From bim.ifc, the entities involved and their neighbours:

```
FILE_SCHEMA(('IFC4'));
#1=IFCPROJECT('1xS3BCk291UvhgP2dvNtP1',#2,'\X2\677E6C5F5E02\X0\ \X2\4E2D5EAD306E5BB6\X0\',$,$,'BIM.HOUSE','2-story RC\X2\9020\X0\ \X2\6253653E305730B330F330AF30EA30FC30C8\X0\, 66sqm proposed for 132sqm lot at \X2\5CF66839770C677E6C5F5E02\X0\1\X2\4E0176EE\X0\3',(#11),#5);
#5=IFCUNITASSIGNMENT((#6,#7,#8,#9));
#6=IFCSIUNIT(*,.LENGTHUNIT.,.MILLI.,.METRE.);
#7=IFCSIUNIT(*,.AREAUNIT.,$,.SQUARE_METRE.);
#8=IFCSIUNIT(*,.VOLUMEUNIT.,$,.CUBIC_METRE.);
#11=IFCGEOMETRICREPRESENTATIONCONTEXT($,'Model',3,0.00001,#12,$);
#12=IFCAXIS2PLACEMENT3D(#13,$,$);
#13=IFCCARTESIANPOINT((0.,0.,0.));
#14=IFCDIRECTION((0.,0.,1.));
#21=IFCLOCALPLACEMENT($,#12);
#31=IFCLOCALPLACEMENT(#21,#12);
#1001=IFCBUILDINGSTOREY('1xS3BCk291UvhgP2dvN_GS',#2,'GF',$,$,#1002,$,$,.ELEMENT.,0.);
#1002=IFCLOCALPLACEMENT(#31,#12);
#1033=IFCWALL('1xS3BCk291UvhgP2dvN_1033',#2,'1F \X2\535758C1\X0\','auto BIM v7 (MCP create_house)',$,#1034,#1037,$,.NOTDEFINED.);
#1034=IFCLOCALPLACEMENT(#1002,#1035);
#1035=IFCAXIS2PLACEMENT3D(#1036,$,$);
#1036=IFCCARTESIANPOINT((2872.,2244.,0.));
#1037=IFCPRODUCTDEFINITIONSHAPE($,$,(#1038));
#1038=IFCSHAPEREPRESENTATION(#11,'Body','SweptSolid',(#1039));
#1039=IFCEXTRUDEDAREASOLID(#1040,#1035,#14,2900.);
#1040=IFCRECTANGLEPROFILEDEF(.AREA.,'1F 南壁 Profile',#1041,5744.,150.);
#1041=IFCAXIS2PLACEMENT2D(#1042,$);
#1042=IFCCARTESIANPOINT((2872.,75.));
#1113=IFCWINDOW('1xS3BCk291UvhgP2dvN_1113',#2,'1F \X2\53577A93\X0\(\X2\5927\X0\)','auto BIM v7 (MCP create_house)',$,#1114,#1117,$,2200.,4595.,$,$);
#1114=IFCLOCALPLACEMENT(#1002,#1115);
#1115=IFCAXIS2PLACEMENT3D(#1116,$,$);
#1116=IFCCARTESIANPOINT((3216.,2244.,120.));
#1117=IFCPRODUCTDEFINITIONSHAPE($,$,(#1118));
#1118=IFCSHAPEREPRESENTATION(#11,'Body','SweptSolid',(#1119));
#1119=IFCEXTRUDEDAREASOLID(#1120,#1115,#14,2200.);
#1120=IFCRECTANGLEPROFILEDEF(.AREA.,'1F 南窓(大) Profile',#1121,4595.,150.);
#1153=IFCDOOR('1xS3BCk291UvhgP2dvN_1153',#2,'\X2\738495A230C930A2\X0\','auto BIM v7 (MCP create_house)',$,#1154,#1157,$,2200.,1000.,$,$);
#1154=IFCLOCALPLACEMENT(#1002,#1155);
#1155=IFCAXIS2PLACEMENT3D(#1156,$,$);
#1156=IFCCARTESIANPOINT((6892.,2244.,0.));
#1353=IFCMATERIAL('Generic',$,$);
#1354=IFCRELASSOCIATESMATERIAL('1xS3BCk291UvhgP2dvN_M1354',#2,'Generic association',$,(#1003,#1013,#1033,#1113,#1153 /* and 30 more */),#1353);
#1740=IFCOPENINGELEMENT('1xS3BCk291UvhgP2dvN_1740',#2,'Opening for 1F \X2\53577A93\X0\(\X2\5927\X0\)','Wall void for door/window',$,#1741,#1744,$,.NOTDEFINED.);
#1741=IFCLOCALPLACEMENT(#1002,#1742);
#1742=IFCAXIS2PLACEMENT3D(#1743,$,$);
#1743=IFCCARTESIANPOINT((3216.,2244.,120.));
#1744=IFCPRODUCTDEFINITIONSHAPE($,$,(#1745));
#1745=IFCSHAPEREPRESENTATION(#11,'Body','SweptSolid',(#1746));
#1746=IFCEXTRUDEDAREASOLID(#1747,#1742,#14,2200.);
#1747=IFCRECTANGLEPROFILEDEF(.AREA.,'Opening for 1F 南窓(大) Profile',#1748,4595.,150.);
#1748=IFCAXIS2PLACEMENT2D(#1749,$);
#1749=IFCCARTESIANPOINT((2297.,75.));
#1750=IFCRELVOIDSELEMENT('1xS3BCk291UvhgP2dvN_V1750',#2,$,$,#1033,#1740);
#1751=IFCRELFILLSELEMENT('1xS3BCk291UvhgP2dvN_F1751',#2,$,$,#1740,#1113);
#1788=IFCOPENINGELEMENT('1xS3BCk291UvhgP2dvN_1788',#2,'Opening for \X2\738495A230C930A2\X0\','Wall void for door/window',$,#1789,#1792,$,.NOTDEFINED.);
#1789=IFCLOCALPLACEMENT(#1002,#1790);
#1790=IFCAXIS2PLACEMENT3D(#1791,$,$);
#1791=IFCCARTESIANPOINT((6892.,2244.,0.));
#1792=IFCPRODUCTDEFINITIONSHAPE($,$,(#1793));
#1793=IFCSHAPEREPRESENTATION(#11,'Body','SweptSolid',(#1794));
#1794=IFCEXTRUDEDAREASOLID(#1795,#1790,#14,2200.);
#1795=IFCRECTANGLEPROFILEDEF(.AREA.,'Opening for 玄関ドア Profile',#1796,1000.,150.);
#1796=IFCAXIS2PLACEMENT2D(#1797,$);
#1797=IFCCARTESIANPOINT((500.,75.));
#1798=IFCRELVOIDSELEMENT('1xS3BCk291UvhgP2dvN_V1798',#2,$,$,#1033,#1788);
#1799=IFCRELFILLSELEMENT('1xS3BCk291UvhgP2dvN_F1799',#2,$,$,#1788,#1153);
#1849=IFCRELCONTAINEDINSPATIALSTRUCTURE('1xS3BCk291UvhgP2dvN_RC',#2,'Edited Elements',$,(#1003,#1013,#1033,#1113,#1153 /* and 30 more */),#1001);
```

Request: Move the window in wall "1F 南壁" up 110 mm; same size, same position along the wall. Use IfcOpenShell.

```python
import numpy as np
import ifcopenshell
import ifcopenshell.api.geometry
import ifcopenshell.util.placement
import ifcopenshell.util.unit

model = ifcopenshell.open("bim.ifc")
unit_scale = ifcopenshell.util.unit.calculate_unit_scale(model)

window = model.by_guid("1xS3BCk291UvhgP2dvN_1113")
opening = window.FillsVoids[0].RelatingOpeningElement
dz = 110.0

shift = np.array([0.0, 0.0, dz])
# The window is not placed relative to its opening, so move both.
for product in (opening, window):
    matrix = ifcopenshell.util.placement.get_local_placement(product.ObjectPlacement)
    matrix[:3, 3] += shift
    ifcopenshell.api.geometry.edit_object_placement(model, product=product, matrix=matrix, is_si=False)

print(f"moved by {dz * unit_scale:+.3f} m")

model.write("bim_edited.ifc")
```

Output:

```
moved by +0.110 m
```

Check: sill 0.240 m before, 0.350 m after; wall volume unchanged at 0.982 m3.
